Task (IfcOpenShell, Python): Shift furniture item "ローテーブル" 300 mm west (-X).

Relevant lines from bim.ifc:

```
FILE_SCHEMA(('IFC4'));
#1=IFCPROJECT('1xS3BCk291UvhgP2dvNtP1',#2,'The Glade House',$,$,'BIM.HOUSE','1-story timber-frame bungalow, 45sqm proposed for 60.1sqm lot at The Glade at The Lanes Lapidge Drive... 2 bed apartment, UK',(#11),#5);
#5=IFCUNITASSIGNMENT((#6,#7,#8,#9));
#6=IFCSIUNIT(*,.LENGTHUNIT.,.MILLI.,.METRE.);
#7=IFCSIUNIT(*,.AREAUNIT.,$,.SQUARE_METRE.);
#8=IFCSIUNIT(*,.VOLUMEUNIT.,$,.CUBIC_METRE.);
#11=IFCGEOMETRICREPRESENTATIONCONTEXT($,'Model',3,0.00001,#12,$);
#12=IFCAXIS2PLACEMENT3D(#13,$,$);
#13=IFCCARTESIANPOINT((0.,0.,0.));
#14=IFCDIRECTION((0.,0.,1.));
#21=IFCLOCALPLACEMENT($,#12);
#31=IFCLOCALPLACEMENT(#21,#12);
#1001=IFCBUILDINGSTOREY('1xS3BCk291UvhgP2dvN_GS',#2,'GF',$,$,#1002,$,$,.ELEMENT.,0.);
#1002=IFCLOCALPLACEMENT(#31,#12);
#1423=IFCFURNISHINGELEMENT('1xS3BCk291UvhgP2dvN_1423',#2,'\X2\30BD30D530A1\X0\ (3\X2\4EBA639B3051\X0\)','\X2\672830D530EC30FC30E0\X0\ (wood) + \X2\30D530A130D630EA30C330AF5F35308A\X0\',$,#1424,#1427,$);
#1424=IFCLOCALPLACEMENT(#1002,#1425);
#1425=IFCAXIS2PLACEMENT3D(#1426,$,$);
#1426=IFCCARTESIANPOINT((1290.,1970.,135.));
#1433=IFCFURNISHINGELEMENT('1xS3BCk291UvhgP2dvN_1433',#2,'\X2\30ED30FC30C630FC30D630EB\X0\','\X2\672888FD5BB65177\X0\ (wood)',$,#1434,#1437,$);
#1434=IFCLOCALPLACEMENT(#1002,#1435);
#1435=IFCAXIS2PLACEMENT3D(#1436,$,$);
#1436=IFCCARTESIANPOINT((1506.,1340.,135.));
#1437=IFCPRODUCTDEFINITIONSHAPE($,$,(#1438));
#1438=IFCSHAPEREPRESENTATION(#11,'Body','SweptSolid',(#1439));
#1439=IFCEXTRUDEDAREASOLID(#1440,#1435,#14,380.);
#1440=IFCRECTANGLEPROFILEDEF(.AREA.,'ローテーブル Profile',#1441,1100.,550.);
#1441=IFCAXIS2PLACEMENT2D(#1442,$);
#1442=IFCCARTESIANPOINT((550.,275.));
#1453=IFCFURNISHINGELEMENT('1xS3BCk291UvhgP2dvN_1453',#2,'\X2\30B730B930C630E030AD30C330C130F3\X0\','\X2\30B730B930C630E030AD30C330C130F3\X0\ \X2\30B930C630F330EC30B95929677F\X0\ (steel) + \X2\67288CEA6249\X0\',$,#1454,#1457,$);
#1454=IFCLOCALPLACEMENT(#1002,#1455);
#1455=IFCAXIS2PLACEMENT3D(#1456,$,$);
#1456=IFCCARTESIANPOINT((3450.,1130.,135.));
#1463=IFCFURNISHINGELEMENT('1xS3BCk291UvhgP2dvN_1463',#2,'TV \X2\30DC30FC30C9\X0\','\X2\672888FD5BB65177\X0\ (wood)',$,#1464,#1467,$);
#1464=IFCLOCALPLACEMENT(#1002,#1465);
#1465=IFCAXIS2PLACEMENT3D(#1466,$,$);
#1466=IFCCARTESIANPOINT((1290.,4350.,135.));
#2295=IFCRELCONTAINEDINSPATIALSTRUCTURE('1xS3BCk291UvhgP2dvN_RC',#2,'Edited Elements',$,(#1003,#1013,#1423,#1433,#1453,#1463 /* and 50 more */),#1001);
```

```python
import ifcopenshell
import ifcopenshell.api.geometry
import ifcopenshell.util.placement

model = ifcopenshell.open("bim.ifc")

item = model.by_guid("1xS3BCk291UvhgP2dvN_1433")
matrix = ifcopenshell.util.placement.get_local_placement(item.ObjectPlacement)
matrix[0, 3] -= 300.0
ifcopenshell.api.geometry.edit_object_placement(model, product=item, matrix=matrix, is_si=False)

print(ifcopenshell.util.placement.get_local_placement(item.ObjectPlacement).round(3) + 0.0)

model.write("bim-out.ifc")
```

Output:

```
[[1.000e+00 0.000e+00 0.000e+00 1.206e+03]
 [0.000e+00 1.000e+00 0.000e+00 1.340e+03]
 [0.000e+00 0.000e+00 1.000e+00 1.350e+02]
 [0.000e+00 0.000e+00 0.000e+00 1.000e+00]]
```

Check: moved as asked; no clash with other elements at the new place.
